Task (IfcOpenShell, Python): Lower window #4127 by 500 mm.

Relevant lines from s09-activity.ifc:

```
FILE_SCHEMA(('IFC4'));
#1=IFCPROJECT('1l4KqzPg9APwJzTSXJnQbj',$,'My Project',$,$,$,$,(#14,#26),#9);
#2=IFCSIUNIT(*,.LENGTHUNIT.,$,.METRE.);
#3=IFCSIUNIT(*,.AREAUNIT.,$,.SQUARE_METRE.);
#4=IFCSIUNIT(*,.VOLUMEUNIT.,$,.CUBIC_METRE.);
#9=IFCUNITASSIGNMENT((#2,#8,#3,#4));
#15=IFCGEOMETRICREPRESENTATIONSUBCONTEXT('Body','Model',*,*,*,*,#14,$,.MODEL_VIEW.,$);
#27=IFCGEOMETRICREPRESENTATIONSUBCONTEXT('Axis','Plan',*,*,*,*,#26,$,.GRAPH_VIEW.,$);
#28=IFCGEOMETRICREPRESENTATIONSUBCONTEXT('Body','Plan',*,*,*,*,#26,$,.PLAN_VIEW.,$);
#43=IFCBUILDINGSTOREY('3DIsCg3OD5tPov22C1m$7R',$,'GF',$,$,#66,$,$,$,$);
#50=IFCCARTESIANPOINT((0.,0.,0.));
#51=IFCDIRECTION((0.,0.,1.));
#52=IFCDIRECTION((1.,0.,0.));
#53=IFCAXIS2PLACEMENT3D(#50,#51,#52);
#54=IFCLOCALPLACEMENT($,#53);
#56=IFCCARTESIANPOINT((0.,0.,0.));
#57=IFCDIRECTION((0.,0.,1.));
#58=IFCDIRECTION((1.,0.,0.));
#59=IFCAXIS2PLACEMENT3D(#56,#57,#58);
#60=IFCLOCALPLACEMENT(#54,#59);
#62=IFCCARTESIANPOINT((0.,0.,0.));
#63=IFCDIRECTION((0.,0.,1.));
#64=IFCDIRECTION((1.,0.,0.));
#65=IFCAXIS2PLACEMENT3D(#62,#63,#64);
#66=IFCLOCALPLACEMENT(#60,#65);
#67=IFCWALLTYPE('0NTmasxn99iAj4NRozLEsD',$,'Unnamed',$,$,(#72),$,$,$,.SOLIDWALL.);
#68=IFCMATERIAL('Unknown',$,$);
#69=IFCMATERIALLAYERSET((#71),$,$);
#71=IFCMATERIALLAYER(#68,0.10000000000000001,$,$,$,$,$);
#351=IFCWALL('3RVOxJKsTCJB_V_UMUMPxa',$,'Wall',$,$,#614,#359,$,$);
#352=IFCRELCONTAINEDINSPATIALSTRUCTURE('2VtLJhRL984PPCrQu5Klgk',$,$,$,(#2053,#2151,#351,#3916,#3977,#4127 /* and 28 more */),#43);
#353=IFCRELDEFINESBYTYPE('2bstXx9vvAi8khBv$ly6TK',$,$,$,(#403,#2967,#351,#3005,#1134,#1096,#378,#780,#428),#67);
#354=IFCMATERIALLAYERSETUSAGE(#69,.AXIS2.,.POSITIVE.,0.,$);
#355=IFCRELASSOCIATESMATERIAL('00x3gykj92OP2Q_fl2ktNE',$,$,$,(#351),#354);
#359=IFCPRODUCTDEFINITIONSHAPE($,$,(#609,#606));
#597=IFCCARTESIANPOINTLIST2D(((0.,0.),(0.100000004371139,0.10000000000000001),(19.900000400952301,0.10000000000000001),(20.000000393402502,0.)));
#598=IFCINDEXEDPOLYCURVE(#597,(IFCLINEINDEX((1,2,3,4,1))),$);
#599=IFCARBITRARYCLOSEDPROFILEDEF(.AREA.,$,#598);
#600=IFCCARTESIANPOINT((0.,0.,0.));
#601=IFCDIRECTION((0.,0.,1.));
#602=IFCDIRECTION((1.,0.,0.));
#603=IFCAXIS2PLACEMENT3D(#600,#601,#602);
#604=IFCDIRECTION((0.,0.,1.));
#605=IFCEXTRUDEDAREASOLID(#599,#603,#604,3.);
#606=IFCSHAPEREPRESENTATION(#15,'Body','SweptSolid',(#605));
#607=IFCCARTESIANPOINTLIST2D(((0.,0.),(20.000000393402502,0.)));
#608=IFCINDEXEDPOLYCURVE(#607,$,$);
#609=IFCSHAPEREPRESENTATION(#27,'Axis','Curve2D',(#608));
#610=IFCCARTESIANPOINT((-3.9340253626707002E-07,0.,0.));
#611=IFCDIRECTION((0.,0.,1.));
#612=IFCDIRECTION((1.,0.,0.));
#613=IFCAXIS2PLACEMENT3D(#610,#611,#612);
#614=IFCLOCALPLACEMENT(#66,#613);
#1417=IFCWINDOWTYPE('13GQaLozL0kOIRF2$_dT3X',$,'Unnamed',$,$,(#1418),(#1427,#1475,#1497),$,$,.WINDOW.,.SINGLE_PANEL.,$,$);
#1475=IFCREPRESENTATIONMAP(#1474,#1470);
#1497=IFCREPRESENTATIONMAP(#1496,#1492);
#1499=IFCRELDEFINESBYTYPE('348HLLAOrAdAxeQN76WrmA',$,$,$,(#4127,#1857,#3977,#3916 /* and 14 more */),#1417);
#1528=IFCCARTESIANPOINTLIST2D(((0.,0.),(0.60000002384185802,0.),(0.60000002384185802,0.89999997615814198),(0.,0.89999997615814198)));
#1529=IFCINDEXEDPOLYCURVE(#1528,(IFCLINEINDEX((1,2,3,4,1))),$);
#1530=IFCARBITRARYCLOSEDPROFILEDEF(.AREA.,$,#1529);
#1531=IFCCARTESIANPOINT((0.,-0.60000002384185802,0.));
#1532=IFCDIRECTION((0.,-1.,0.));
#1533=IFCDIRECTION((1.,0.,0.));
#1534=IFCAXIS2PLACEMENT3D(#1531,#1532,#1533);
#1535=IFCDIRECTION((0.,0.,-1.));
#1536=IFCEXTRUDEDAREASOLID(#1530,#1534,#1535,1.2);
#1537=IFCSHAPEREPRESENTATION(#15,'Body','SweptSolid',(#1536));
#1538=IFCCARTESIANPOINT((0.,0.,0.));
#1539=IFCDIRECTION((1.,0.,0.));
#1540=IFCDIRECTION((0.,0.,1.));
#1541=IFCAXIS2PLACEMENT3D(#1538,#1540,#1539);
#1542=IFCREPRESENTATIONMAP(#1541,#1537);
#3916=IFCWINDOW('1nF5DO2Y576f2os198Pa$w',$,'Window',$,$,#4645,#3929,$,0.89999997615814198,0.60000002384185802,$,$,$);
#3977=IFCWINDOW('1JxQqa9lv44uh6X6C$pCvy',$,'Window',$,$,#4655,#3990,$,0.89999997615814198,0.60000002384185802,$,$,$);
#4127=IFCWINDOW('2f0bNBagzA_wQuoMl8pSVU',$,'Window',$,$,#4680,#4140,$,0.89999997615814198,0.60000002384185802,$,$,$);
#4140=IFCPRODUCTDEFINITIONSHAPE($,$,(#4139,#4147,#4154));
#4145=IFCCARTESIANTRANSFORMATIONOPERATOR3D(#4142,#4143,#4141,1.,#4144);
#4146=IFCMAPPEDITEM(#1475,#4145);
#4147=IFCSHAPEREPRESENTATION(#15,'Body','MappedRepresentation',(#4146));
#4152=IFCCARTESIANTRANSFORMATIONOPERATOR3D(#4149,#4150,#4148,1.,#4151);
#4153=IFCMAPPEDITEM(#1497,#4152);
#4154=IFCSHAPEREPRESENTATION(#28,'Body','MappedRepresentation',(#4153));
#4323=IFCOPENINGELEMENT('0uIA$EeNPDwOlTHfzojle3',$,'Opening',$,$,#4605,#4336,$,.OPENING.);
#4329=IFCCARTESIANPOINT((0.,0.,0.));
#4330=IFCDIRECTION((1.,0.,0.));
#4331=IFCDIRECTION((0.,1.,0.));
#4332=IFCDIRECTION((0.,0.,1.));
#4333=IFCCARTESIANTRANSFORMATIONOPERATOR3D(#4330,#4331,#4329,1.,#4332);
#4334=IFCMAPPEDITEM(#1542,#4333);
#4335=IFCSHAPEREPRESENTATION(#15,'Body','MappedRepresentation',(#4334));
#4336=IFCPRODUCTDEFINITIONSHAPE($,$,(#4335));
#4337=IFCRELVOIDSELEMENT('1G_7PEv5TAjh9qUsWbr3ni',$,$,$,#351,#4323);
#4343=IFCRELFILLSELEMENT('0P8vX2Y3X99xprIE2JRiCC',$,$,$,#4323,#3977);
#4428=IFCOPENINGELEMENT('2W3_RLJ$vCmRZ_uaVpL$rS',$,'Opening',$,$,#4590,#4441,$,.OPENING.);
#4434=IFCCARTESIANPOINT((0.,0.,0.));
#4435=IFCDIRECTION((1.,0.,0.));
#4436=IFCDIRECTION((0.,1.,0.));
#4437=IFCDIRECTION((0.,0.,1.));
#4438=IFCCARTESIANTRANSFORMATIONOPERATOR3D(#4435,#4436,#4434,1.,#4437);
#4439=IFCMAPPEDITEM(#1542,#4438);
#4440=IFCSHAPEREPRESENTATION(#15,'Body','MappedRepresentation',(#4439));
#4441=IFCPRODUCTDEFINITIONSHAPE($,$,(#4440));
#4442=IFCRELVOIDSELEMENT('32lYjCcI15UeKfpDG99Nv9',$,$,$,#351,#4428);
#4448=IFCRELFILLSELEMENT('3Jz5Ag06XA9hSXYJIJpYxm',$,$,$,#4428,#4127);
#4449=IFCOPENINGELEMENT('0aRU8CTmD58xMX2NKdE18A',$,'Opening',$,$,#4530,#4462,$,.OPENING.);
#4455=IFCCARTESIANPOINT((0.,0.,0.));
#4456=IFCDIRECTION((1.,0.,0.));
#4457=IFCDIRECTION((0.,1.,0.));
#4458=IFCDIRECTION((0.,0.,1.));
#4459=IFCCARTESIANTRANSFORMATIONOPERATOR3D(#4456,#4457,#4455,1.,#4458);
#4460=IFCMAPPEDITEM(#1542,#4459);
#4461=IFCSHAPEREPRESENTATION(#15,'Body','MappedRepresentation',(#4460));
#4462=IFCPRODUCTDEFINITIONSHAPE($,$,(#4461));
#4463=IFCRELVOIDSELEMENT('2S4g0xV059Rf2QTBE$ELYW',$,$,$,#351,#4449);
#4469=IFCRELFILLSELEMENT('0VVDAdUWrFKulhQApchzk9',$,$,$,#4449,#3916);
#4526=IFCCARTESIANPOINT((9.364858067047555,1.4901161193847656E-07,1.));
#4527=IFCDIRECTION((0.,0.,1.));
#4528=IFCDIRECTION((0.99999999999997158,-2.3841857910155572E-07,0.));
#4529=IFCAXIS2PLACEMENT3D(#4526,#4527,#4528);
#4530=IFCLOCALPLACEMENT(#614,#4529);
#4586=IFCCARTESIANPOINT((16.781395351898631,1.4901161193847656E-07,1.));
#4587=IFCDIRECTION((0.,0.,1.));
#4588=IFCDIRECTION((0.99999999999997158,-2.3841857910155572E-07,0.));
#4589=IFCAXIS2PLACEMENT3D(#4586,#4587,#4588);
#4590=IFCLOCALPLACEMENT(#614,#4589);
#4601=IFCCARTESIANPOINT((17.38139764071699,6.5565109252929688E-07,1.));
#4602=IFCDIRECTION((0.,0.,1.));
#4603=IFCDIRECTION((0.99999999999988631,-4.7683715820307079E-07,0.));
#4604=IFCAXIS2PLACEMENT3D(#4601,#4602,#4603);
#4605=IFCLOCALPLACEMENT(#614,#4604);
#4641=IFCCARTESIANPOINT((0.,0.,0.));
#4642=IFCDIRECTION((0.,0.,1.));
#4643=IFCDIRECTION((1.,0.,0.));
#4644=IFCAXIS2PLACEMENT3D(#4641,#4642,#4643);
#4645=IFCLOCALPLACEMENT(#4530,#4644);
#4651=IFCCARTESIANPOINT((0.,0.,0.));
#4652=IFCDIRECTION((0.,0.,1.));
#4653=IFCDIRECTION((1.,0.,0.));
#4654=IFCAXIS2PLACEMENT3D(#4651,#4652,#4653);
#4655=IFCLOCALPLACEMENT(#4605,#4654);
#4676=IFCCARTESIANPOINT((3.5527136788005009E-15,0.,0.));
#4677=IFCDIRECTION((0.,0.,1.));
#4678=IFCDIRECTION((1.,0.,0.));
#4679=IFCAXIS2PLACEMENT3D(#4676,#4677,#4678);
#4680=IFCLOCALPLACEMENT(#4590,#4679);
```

```python
import numpy as np
import ifcopenshell
import ifcopenshell.api.geometry
import ifcopenshell.util.placement
import ifcopenshell.util.unit

model = ifcopenshell.open("s09-activity.ifc")
unit_scale = ifcopenshell.util.unit.calculate_unit_scale(model)

window = model.by_id(4127)
opening = window.FillsVoids[0].RelatingOpeningElement
dz = -0.5

shift = np.array([0.0, 0.0, dz])
# The window is placed relative to its opening, so it follows when the opening moves.
matrix = ifcopenshell.util.placement.get_local_placement(opening.ObjectPlacement)
matrix[:3, 3] += shift
ifcopenshell.api.geometry.edit_object_placement(
    model, product=opening, matrix=matrix, is_si=False, should_transform_children=True
)

print(f"moved by {dz * unit_scale:+.3f} m")

model.write("s09-activity_v2.ifc")
```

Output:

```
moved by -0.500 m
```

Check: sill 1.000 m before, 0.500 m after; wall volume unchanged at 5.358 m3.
